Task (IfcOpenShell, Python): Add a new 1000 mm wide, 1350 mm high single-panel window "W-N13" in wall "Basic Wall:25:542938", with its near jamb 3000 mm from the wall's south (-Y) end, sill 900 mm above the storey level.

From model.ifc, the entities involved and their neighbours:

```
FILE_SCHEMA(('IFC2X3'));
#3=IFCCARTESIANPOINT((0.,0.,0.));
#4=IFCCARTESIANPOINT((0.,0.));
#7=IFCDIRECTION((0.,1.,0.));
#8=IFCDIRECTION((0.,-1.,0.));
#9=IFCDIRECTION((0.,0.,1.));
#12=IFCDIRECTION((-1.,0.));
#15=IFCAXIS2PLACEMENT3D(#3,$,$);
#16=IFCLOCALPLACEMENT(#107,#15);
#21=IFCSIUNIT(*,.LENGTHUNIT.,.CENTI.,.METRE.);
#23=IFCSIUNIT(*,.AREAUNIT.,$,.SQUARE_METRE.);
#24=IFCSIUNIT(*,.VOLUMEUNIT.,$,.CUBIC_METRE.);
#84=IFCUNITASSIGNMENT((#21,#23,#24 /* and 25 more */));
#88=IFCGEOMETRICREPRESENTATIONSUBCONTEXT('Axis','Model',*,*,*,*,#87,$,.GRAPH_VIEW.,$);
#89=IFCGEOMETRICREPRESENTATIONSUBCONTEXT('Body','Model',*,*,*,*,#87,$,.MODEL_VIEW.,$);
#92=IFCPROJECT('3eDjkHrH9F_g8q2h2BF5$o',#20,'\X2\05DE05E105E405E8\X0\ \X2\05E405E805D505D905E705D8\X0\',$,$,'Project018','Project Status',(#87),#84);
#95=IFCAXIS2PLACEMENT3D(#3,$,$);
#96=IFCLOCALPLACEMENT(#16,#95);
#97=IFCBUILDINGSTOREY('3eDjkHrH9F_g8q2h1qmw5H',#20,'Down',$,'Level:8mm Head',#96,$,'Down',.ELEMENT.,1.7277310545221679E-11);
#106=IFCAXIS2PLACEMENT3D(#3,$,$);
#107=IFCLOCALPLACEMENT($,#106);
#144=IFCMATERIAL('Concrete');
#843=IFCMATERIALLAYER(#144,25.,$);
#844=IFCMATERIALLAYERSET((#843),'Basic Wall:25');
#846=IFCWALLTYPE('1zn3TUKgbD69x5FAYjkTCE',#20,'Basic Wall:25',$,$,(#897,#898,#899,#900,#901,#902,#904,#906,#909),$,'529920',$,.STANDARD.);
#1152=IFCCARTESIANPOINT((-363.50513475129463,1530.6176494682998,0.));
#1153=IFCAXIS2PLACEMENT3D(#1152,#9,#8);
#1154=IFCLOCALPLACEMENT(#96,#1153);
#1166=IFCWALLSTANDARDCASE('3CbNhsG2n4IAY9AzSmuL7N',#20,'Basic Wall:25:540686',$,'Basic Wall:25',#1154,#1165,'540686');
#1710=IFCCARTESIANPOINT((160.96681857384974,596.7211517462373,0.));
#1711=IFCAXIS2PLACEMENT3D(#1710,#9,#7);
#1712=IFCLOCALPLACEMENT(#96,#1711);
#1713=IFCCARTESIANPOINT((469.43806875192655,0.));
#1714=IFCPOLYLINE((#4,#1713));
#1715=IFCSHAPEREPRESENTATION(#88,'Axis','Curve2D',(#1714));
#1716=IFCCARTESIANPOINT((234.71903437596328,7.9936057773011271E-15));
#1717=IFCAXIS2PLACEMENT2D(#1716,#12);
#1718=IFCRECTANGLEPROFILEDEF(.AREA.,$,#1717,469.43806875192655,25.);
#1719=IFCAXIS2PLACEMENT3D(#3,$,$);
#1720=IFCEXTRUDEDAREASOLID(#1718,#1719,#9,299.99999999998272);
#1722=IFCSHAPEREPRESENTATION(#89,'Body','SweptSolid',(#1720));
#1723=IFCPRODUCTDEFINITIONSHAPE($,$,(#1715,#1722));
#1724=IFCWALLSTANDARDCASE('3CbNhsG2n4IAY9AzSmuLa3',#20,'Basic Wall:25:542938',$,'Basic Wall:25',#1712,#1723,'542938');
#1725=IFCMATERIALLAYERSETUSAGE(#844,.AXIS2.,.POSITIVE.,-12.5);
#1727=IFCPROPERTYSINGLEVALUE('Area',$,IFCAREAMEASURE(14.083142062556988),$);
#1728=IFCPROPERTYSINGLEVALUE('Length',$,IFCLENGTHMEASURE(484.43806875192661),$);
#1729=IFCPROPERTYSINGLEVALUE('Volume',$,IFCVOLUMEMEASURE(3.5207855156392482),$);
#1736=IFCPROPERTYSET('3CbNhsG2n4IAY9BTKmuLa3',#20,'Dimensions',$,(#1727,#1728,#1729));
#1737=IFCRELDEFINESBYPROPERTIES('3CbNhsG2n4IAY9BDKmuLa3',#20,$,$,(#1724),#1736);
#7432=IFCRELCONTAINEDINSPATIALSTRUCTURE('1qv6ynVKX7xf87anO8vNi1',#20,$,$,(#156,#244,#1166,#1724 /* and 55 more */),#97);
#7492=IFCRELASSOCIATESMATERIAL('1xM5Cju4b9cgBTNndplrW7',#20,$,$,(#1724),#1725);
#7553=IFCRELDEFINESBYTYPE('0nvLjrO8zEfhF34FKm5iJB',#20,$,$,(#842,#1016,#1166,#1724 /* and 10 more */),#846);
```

```python
import numpy as np
import ifcopenshell
import ifcopenshell.api.feature
import ifcopenshell.api.geometry
import ifcopenshell.api.pset
import ifcopenshell.api.root
import ifcopenshell.api.spatial
import ifcopenshell.api.type
import ifcopenshell.geom
import ifcopenshell.util.element
import ifcopenshell.util.placement
import ifcopenshell.util.representation
import ifcopenshell.util.shape
import ifcopenshell.util.unit

model = ifcopenshell.open("model.ifc")
unit_scale = ifcopenshell.util.unit.calculate_unit_scale(model)
area_scale = ifcopenshell.util.unit.calculate_unit_scale(model, "AREAUNIT")
volume_scale = ifcopenshell.util.unit.calculate_unit_scale(model, "VOLUMEUNIT")
settings = ifcopenshell.geom.settings()


def volume(element):
    """Net volume in cubic metres, openings subtracted."""
    shape = ifcopenshell.geom.create_shape(settings, element)
    return ifcopenshell.util.shape.get_volume(shape.geometry)


wall = model.by_guid("3CbNhsG2n4IAY9AzSmuLa3")
storey = ifcopenshell.util.element.get_container(wall, ifc_class="IfcBuildingStorey")
context = ifcopenshell.util.representation.get_context(model, "Model", "Body", "MODEL_VIEW")
before = volume(wall)

width, height, from_end, sill = 1, 1.35, 3, 0.9  # metres

# The wall runs along its own X axis, and the end named is its -X end.
wall_shape = ifcopenshell.geom.create_shape(settings, wall)
x, y, z = ifcopenshell.util.shape.get_vertices(wall_shape.geometry).T
start = x.min() + from_end
face, thickness = float(y.min()), float(y.max() - y.min())
wall_matrix = ifcopenshell.util.placement.get_local_placement(wall.ObjectPlacement)
level = ifcopenshell.util.placement.get_local_placement(storey.ObjectPlacement)[2, 3]


def in_wall(x, y):
    """Placement at x, y metres in the wall's axes, at sill height."""
    matrix = wall_matrix.copy()
    matrix[:, 3] = wall_matrix @ np.array([x / unit_scale, y / unit_scale, 0.0, 1.0])
    matrix[2, 3] = level + sill / unit_scale
    return matrix


# Opening: a box that overshoots both wall faces by 50 mm.
opening = ifcopenshell.api.root.create_entity(model, ifc_class="IfcOpeningElement")
box = ifcopenshell.api.geometry.add_wall_representation(
    model, context=context, length=width, height=height, thickness=thickness + 0.1
)
ifcopenshell.api.geometry.assign_representation(model, product=opening, representation=box)
ifcopenshell.api.geometry.edit_object_placement(model, product=opening, matrix=in_wall(start, face - 0.05), is_si=False)
ifcopenshell.api.feature.add_feature(model, feature=opening, element=wall)

window = ifcopenshell.api.root.create_entity(model, ifc_class="IfcWindow", name="W-N13")
window.OverallWidth, window.OverallHeight = width / unit_scale, height / unit_scale
body = ifcopenshell.api.geometry.add_window_representation(
    model,
    context=context,
    overall_width=window.OverallWidth,
    overall_height=window.OverallHeight,
    partition_type="SINGLE_PANEL",
)
ifcopenshell.api.geometry.assign_representation(model, product=window, representation=body)
ifcopenshell.api.spatial.assign_container(model, products=[window], relating_structure=storey)
fills = ifcopenshell.api.feature.add_filling(model, opening=opening, element=window)
fills.OwnerHistory = window.OwnerHistory  # required in IFC2X3

# IFC2X3 keeps the operation on the window style.
style = ifcopenshell.api.root.create_entity(model, ifc_class="IfcWindowStyle", name="W-N13")
style.OperationType, style.ConstructionType = "SINGLE_PANEL", "NOTDEFINED"
style.ParameterTakesPrecedence = style.Sizeable = False
ifcopenshell.api.type.assign_type(model, related_objects=[window], relating_type=style)

# Centre the window in the wall's thickness.
ifcopenshell.api.geometry.edit_object_placement(model, product=window, matrix=in_wall(start, face), is_si=False)
window_shape = ifcopenshell.geom.create_shape(settings, window)
depth = ifcopenshell.util.shape.get_vertices(window_shape.geometry)[:, 1]
offset = face + thickness / 2 - (depth.min() + depth.max()) / 2
ifcopenshell.api.geometry.edit_object_placement(model, product=window, matrix=in_wall(start, offset), is_si=False)

after = volume(wall)

# Update the wall's stored quantities.
pset = model.by_id(ifcopenshell.util.element.get_pset(wall, "Dimensions", should_inherit=False)["id"])
ifcopenshell.api.pset.edit_pset(model, pset=pset, properties={
    "Area": model.create_entity("IfcAreaMeasure", after / thickness / area_scale),
    "Volume": model.create_entity("IfcVolumeMeasure", after / volume_scale),
})

print(f"wall volume {before:.3f} -> {after:.3f} m3")

model.write("model_rev.ifc")
```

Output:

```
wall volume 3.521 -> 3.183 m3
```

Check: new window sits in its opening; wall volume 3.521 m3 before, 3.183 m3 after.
